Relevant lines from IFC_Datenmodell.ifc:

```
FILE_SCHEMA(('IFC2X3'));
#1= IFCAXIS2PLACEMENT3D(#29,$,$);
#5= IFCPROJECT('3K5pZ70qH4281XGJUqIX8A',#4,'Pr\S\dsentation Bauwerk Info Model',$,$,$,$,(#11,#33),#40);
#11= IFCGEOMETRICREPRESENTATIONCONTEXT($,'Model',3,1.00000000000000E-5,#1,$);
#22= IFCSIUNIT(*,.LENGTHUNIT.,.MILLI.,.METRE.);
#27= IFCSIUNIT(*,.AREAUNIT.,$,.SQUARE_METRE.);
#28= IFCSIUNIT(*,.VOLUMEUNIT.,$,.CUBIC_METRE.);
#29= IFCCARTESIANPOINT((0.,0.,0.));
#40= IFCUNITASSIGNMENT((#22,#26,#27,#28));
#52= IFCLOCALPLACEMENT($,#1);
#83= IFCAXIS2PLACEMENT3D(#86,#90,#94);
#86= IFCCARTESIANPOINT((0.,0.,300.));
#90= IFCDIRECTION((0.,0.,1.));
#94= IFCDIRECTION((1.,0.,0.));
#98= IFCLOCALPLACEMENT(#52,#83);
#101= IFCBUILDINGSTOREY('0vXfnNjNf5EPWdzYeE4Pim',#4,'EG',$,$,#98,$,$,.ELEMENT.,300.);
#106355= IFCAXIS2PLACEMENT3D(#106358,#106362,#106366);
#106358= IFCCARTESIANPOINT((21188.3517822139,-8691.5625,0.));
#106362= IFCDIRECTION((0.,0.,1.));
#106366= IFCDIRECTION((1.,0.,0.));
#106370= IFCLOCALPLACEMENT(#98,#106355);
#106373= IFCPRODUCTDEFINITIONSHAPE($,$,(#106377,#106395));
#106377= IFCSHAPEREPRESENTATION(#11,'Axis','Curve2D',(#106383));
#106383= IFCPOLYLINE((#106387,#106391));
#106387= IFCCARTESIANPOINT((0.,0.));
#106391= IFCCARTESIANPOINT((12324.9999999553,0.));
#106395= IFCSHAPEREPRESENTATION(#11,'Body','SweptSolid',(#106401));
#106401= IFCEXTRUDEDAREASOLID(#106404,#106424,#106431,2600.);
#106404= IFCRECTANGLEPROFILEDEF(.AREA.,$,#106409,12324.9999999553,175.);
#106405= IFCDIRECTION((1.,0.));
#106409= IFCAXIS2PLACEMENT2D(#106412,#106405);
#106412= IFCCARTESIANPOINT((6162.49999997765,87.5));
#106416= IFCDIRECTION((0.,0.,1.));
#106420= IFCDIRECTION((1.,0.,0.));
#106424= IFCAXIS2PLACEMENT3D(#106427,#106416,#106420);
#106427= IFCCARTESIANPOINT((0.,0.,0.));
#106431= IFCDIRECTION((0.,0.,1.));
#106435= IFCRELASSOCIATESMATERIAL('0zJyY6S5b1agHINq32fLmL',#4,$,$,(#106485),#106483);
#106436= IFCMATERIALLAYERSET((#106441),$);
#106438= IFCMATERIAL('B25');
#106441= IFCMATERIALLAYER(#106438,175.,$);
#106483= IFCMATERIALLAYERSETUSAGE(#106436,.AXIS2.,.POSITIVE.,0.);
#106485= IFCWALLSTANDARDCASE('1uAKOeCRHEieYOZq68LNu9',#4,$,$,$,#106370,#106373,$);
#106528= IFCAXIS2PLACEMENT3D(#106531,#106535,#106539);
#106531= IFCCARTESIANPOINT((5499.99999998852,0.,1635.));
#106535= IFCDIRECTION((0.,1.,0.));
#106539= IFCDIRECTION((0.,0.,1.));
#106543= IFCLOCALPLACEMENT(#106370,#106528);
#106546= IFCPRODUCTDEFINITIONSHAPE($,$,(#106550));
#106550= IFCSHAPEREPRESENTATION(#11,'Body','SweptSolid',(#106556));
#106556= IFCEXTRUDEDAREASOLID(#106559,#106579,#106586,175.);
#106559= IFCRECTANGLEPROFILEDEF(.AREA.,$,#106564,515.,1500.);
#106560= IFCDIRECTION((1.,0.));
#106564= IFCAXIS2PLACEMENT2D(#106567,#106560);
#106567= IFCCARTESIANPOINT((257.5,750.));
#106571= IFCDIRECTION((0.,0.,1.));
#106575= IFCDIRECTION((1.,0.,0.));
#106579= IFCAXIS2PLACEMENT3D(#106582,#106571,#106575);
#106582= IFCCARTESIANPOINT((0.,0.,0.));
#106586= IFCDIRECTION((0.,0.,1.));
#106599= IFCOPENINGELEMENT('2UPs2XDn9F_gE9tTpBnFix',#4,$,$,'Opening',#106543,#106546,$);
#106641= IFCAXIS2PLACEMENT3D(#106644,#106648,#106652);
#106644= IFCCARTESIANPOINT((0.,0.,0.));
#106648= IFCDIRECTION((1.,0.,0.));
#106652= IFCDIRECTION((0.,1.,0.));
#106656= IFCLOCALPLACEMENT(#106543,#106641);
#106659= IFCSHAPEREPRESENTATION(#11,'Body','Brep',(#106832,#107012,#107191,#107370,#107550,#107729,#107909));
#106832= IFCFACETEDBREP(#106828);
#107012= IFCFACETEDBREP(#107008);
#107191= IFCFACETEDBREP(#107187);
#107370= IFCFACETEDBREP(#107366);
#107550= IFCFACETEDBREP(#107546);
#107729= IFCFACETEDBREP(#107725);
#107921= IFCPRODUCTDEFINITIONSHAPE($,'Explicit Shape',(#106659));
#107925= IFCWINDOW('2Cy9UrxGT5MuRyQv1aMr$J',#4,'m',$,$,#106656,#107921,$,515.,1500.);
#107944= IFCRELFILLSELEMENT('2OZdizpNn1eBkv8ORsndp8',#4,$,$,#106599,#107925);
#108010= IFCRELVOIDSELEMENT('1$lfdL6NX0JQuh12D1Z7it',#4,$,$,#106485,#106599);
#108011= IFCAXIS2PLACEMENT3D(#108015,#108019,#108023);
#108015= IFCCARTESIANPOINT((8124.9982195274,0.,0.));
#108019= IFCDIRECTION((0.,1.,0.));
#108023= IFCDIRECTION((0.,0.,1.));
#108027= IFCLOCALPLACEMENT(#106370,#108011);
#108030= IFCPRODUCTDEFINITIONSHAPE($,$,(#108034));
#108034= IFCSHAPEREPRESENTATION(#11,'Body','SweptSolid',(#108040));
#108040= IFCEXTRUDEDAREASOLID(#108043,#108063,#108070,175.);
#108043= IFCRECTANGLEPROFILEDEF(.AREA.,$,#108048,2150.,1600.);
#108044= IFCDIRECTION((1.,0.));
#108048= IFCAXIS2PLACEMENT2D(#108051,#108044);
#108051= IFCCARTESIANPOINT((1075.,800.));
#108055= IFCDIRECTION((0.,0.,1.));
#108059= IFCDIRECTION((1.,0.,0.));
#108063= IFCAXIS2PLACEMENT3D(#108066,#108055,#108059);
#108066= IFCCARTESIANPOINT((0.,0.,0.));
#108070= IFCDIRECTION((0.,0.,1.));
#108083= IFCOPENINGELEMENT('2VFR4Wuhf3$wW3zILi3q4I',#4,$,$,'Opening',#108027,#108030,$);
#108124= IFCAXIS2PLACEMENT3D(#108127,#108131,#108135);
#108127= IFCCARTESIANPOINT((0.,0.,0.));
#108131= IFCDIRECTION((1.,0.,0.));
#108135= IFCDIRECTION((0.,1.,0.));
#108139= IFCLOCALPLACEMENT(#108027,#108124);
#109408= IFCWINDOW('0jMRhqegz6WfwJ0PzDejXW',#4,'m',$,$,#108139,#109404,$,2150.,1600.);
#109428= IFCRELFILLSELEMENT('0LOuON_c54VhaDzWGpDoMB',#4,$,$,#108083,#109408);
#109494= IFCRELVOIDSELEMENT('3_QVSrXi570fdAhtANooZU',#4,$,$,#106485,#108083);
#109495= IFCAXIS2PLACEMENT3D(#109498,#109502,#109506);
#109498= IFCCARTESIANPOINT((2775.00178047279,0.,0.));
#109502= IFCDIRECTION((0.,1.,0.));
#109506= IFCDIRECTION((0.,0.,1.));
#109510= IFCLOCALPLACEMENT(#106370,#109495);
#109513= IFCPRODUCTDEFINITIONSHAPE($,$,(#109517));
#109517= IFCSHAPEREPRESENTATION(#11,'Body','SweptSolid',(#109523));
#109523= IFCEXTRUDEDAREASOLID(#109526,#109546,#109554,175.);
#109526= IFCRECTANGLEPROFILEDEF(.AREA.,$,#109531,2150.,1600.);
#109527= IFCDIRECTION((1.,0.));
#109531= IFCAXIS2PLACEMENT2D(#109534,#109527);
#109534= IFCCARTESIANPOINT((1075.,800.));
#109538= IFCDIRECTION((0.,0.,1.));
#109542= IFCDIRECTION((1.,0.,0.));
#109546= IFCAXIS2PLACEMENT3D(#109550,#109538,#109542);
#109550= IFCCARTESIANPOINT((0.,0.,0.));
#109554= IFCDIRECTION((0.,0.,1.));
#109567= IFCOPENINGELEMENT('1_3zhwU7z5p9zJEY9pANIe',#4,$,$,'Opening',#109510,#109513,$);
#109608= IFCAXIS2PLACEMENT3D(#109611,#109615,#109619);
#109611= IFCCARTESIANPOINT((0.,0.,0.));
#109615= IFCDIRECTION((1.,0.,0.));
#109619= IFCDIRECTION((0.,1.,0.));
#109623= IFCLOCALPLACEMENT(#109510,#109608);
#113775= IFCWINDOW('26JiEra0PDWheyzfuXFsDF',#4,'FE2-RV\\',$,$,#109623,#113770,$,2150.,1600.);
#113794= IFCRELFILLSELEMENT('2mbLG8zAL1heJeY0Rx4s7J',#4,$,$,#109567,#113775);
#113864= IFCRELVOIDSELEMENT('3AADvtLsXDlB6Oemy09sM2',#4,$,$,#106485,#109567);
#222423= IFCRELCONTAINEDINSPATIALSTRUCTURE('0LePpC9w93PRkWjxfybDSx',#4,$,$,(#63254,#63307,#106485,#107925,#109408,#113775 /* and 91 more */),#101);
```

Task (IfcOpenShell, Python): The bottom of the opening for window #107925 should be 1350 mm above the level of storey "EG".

```python
import numpy as np
import ifcopenshell
import ifcopenshell.api.geometry
import ifcopenshell.geom
import ifcopenshell.util.element
import ifcopenshell.util.placement
import ifcopenshell.util.shape
import ifcopenshell.util.unit

model = ifcopenshell.open("IFC_Datenmodell.ifc")
unit_scale = ifcopenshell.util.unit.calculate_unit_scale(model)

window = model.by_guid("2Cy9UrxGT5MuRyQv1aMr$J")
opening = window.FillsVoids[0].RelatingOpeningElement
storey = ifcopenshell.util.element.get_container(window, ifc_class="IfcBuildingStorey")
level = ifcopenshell.util.placement.get_local_placement(storey.ObjectPlacement)[2, 3]

# The opening's origin need not be at the sill, so measure its lowest point.
shape = ifcopenshell.geom.create_shape(ifcopenshell.geom.settings(), opening)
bottom = ifcopenshell.util.shape.get_shape_bottom_elevation(shape, shape.geometry) / unit_scale
dz = level + 1.35 / unit_scale - bottom

shift = np.array([0.0, 0.0, dz])
# The window is placed relative to its opening, so it follows when the opening moves.
matrix = ifcopenshell.util.placement.get_local_placement(opening.ObjectPlacement)
matrix[:3, 3] += shift
ifcopenshell.api.geometry.edit_object_placement(
    model, product=opening, matrix=matrix, is_si=False, should_transform_children=True
)

print(f"moved by {dz * unit_scale:+.3f} m")

model.write("IFC_Datenmodell-out.ifc")
```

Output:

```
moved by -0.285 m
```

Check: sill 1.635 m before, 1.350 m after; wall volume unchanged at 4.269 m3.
